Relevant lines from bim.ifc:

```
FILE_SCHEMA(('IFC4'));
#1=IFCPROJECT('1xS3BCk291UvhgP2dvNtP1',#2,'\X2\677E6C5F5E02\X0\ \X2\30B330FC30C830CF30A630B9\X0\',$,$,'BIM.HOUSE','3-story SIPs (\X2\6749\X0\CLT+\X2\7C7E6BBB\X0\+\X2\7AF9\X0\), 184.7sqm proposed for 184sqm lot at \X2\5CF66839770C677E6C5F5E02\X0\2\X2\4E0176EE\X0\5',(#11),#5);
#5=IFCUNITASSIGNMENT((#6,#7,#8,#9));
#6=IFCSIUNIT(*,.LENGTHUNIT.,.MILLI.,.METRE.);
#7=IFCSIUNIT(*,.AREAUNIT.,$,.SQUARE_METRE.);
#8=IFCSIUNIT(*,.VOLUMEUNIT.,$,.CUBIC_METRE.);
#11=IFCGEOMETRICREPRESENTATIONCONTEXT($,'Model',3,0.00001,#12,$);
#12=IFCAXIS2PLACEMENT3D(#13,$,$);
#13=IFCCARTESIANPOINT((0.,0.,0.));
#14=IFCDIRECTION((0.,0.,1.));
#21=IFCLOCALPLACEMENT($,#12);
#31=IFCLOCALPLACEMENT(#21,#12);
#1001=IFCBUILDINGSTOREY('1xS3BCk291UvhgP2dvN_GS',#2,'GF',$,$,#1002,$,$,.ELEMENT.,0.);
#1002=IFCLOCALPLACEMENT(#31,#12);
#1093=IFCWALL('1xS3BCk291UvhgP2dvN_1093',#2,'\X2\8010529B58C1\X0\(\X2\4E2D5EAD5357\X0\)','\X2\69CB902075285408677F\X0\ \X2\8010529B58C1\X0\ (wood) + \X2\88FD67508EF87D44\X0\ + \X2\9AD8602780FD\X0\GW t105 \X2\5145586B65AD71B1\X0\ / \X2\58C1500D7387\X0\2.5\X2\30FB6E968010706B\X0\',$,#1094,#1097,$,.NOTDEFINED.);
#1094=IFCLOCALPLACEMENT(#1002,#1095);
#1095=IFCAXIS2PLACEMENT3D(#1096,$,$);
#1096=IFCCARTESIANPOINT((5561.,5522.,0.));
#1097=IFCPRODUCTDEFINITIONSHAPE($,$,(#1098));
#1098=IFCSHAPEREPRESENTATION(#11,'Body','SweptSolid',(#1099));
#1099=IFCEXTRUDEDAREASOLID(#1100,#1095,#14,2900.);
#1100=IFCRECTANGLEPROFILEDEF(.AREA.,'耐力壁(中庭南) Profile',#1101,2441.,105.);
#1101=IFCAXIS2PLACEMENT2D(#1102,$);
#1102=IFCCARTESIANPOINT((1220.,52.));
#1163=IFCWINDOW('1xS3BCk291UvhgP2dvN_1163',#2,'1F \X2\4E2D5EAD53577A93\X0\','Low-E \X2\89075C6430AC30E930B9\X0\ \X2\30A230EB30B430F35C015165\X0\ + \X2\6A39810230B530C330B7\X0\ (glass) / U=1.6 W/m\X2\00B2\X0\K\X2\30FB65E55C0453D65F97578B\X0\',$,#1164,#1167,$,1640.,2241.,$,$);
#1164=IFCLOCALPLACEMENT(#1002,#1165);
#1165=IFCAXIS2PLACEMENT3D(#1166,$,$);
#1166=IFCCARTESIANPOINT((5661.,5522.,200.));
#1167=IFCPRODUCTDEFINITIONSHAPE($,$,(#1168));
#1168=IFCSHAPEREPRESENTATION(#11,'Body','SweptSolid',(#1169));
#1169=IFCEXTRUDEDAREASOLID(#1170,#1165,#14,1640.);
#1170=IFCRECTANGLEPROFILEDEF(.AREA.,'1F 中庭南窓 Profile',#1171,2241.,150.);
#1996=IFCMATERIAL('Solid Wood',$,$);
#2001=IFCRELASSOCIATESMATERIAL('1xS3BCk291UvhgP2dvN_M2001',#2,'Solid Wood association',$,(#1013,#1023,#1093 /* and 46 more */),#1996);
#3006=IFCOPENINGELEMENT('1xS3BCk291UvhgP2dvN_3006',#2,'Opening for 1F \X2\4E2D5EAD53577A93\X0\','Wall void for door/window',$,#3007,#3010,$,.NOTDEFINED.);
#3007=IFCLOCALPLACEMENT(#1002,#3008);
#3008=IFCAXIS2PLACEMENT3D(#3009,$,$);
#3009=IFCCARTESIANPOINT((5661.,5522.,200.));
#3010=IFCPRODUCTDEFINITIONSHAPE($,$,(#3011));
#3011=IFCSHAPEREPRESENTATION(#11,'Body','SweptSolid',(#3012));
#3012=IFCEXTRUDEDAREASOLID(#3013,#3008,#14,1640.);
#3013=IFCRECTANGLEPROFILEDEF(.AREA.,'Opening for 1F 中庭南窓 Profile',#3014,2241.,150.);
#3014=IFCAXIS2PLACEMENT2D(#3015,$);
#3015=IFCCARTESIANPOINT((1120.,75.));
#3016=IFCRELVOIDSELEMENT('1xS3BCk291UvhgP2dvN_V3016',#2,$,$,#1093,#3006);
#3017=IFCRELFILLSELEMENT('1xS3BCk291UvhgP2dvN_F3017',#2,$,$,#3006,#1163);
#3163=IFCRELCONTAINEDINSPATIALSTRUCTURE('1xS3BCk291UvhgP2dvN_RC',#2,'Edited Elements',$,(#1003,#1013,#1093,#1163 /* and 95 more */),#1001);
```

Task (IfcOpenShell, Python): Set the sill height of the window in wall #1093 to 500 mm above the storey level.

```python
import numpy as np
import ifcopenshell
import ifcopenshell.api.geometry
import ifcopenshell.geom
import ifcopenshell.util.element
import ifcopenshell.util.placement
import ifcopenshell.util.shape
import ifcopenshell.util.unit

model = ifcopenshell.open("bim.ifc")
unit_scale = ifcopenshell.util.unit.calculate_unit_scale(model)

window = model.by_id(1163)
opening = window.FillsVoids[0].RelatingOpeningElement
storey = ifcopenshell.util.element.get_container(window, ifc_class="IfcBuildingStorey")
level = ifcopenshell.util.placement.get_local_placement(storey.ObjectPlacement)[2, 3]

# The opening's origin need not be at the sill, so measure its lowest point.
shape = ifcopenshell.geom.create_shape(ifcopenshell.geom.settings(), opening)
bottom = ifcopenshell.util.shape.get_shape_bottom_elevation(shape, shape.geometry) / unit_scale
dz = level + 500.0 - bottom

shift = np.array([0.0, 0.0, dz])
# The window is not placed relative to its opening, so move both.
for product in (opening, window):
    matrix = ifcopenshell.util.placement.get_local_placement(product.ObjectPlacement)
    matrix[:3, 3] += shift
    ifcopenshell.api.geometry.edit_object_placement(model, product=product, matrix=matrix, is_si=False)

print(f"moved by {dz * unit_scale:+.3f} m")

model.write("bim_v2.ifc")
```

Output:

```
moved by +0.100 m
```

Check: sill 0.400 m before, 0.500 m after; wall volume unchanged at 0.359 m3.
